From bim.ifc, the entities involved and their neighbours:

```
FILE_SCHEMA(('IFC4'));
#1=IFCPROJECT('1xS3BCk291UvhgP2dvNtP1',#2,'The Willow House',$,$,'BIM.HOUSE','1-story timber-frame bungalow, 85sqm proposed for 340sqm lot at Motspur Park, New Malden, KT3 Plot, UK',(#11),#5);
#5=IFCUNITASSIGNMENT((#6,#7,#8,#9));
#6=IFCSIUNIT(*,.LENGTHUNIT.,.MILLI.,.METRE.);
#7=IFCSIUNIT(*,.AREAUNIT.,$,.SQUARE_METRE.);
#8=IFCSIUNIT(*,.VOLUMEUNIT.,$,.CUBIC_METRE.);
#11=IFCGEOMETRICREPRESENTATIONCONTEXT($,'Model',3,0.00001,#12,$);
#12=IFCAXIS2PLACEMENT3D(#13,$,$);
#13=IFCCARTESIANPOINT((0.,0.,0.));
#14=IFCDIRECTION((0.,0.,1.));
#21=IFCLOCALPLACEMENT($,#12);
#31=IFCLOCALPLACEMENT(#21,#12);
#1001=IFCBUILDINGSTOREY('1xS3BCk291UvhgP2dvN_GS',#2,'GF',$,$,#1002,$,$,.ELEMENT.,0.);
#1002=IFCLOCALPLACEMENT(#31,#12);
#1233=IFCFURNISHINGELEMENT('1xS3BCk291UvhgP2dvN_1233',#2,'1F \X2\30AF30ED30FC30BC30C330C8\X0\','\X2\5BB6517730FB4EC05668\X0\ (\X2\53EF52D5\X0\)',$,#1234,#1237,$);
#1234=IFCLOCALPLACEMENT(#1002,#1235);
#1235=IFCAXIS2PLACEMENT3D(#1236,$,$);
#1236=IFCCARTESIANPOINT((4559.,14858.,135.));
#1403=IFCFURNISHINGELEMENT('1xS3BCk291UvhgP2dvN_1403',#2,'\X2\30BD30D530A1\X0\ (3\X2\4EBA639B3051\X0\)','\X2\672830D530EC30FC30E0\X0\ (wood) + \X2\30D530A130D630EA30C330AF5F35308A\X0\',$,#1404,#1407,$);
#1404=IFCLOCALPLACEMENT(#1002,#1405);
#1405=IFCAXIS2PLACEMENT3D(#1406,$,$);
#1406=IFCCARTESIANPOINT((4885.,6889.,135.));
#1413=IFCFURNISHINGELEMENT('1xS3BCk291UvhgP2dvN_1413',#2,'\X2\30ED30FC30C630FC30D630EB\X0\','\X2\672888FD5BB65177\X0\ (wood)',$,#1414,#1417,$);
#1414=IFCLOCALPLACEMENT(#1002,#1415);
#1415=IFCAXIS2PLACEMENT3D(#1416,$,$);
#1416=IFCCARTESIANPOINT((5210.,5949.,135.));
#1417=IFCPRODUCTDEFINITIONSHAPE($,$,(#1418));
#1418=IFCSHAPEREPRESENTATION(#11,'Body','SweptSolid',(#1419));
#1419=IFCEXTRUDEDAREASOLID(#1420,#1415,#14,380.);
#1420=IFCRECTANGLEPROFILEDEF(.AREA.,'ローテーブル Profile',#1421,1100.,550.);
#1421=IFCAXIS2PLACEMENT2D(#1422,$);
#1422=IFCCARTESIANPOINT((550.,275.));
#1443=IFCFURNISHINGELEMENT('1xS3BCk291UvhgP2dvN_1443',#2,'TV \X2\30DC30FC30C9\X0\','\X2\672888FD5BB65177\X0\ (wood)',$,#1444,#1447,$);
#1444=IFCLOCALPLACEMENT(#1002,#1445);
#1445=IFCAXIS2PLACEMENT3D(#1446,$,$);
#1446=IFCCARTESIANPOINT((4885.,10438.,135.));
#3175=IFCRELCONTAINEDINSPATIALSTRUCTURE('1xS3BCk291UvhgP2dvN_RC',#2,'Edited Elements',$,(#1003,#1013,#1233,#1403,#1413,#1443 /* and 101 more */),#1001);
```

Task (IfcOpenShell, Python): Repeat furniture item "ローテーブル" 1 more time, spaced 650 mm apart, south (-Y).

```python
import numpy as np
import ifcopenshell
import ifcopenshell.api.geometry
import ifcopenshell.api.root
import ifcopenshell.util.element
import ifcopenshell.util.placement
import ifcopenshell.util.unit

model = ifcopenshell.open("bim.ifc")
unit_scale = ifcopenshell.util.unit.calculate_unit_scale(model)


def reuse_history(source, copy):
    """copy_class also copies each property set's owner history, people and application; keep the originals."""
    for rel in copy.IsDefinedBy:
        if rel.is_a("IfcRelDefinesByProperties") and (history := rel.RelatingPropertyDefinition.OwnerHistory):
            rel.RelatingPropertyDefinition.OwnerHistory = source.OwnerHistory
            ifcopenshell.util.element.remove_deep2(model, history)


source = model.by_guid("1xS3BCk291UvhgP2dvN_1413")
base = ifcopenshell.util.placement.get_local_placement(source.ObjectPlacement)
step = np.array([0.0, -1.0, 0.0]) * 0.65 / unit_scale

for i in range(1, 2):
    copy = ifcopenshell.api.root.copy_class(model, product=source)
    copy.Representation = ifcopenshell.util.element.copy_deep(
        model, source.Representation, exclude=["IfcGeometricRepresentationContext", "IfcRepresentationMap"]
    )
    reuse_history(source, copy)
    matrix = base.copy()
    matrix[:3, 3] += i * step
    print("added at", matrix[:3, 3].round(3) + 0.0)
    ifcopenshell.api.geometry.edit_object_placement(model, product=copy, matrix=matrix, is_si=False)

model.write("bim-out.ifc")
```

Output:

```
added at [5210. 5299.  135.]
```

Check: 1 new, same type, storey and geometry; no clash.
